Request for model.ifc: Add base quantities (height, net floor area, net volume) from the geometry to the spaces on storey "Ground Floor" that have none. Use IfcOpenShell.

First a look at what the model holds.

```python
import ifcopenshell
import ifcopenshell.util.element
import ifcopenshell.util.unit

model = ifcopenshell.open("model.ifc")
print(model.schema)
for unit_type in ("LENGTHUNIT", "AREAUNIT", "VOLUMEUNIT"):
    print(unit_type, ifcopenshell.util.unit.calculate_unit_scale(model, unit_type))
storey = next(s for s in model.by_type("IfcBuildingStorey") if s.Name == "Ground Floor")
spaces = [e for e in ifcopenshell.util.element.get_decomposition(storey) if e.is_a("IfcSpace")]
for e in sorted(spaces, key=lambda e: e.id()):
    print(e.id(), e.is_a(), e.Name, list(ifcopenshell.util.element.get_psets(e, qtos_only=True)), sep=" | ")
```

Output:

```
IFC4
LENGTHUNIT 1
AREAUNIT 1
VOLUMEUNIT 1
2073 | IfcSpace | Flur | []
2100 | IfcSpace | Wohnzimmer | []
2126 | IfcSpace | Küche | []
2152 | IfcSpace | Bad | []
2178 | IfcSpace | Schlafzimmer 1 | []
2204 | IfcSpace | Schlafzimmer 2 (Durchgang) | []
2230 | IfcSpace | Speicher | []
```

```python
import ifcopenshell
import ifcopenshell.api.pset
import ifcopenshell.geom
import ifcopenshell.util.element
import ifcopenshell.util.shape
import ifcopenshell.util.unit

model = ifcopenshell.open("model.ifc")
unit_scale = ifcopenshell.util.unit.calculate_unit_scale(model)
area_scale = ifcopenshell.util.unit.calculate_unit_scale(model, "AREAUNIT")
volume_scale = ifcopenshell.util.unit.calculate_unit_scale(model, "VOLUMEUNIT")
settings = ifcopenshell.geom.settings()

storey = next(s for s in model.by_type("IfcBuildingStorey") if s.Name == "Ground Floor")
spaces = [e for e in ifcopenshell.util.element.get_decomposition(storey) if e.is_a("IfcSpace")]

for e in sorted(spaces, key=lambda e: e.id()):
    if ifcopenshell.util.element.get_psets(e, qtos_only=True, should_inherit=False):
        continue
    # Geometry comes back in metres, in the element's own axes.
    shape = ifcopenshell.geom.create_shape(settings, e)
    values = {
        "Height": ifcopenshell.util.shape.get_z(shape.geometry) / unit_scale,
        "NetFloorArea": ifcopenshell.util.shape.get_footprint_area(shape.geometry) / area_scale,
        "NetVolume": ifcopenshell.util.shape.get_volume(shape.geometry) / volume_scale,
    }
    qto = ifcopenshell.api.pset.add_qto(model, product=e, name="Qto_SpaceBaseQuantities")
    ifcopenshell.api.pset.edit_qto(model, qto=qto, properties=values)
    print(e.id(), {k: round(v, 3) for k, v in values.items()})

model.write("model_v2.ifc")
```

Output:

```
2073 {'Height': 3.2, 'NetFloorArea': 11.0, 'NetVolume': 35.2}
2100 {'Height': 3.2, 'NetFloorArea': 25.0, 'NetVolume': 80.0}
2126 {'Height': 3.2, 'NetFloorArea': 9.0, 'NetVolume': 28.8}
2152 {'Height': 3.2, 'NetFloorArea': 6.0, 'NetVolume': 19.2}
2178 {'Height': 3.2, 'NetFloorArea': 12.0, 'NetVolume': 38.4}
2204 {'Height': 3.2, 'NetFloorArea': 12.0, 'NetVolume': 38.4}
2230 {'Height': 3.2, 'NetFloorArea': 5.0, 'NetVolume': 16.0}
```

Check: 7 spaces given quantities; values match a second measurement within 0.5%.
